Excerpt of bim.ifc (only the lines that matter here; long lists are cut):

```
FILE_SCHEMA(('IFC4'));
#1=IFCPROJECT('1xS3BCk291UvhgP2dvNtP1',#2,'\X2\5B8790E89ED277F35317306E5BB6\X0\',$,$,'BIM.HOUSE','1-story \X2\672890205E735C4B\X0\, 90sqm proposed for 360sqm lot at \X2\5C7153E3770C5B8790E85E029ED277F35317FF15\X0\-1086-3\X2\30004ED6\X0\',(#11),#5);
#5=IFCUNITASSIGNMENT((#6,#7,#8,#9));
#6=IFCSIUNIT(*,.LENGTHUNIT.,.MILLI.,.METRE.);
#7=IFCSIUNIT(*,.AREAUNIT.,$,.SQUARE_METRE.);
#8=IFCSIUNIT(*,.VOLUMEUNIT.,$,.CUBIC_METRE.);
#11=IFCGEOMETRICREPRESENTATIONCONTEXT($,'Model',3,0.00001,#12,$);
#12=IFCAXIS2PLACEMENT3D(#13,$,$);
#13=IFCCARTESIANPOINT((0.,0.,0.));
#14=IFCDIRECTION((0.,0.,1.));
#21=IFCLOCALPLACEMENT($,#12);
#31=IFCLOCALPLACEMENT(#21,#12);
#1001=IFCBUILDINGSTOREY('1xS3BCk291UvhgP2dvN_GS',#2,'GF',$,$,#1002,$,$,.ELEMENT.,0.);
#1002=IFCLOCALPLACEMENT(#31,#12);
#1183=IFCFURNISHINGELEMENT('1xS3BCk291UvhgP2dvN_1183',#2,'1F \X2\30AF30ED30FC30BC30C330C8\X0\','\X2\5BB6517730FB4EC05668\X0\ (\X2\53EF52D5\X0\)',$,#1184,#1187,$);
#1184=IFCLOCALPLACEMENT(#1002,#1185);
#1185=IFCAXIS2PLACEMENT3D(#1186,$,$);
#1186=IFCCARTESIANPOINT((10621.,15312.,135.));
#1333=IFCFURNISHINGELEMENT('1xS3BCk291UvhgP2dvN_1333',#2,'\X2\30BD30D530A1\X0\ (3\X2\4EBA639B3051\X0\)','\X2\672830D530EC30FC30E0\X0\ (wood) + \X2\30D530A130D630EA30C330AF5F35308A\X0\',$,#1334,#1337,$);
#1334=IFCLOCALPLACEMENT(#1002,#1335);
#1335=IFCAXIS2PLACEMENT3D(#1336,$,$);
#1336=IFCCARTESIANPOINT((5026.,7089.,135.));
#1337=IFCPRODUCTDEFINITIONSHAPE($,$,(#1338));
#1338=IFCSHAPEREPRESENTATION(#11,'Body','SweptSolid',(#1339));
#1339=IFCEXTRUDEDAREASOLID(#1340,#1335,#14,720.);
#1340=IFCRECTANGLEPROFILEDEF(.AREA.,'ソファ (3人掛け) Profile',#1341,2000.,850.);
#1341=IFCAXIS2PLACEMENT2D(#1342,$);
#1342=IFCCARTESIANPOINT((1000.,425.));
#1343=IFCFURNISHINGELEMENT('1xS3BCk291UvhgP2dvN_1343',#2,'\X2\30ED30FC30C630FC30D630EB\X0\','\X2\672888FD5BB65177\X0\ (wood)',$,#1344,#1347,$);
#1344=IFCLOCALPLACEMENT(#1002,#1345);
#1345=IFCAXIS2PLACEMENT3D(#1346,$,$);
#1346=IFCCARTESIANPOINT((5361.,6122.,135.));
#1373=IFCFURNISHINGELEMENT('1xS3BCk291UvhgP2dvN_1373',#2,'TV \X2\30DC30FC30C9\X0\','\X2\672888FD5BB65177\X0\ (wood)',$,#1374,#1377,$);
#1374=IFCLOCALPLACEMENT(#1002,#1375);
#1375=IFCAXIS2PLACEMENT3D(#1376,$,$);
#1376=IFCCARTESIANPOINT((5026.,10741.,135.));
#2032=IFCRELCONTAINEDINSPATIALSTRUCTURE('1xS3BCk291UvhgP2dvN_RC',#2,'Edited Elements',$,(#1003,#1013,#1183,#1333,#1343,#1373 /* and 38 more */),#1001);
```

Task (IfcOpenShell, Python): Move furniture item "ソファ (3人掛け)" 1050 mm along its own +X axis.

```python
import ifcopenshell
import ifcopenshell.api.geometry
import ifcopenshell.util.placement
import ifcopenshell.util.unit

model = ifcopenshell.open("bim.ifc")
unit_scale = ifcopenshell.util.unit.calculate_unit_scale(model)

item = model.by_id(1333)
matrix = ifcopenshell.util.placement.get_local_placement(item.ObjectPlacement)
matrix[:3, 3] += matrix[:3, 0] * 1.05 / unit_scale
ifcopenshell.api.geometry.edit_object_placement(model, product=item, matrix=matrix, is_si=False)

print(ifcopenshell.util.placement.get_local_placement(item.ObjectPlacement).round(3) + 0.0)

model.write("bim_rev.ifc")
```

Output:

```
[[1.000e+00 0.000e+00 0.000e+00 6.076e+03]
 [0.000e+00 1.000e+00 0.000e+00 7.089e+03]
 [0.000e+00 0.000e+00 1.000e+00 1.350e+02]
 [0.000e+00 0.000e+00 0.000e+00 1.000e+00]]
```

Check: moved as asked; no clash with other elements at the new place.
